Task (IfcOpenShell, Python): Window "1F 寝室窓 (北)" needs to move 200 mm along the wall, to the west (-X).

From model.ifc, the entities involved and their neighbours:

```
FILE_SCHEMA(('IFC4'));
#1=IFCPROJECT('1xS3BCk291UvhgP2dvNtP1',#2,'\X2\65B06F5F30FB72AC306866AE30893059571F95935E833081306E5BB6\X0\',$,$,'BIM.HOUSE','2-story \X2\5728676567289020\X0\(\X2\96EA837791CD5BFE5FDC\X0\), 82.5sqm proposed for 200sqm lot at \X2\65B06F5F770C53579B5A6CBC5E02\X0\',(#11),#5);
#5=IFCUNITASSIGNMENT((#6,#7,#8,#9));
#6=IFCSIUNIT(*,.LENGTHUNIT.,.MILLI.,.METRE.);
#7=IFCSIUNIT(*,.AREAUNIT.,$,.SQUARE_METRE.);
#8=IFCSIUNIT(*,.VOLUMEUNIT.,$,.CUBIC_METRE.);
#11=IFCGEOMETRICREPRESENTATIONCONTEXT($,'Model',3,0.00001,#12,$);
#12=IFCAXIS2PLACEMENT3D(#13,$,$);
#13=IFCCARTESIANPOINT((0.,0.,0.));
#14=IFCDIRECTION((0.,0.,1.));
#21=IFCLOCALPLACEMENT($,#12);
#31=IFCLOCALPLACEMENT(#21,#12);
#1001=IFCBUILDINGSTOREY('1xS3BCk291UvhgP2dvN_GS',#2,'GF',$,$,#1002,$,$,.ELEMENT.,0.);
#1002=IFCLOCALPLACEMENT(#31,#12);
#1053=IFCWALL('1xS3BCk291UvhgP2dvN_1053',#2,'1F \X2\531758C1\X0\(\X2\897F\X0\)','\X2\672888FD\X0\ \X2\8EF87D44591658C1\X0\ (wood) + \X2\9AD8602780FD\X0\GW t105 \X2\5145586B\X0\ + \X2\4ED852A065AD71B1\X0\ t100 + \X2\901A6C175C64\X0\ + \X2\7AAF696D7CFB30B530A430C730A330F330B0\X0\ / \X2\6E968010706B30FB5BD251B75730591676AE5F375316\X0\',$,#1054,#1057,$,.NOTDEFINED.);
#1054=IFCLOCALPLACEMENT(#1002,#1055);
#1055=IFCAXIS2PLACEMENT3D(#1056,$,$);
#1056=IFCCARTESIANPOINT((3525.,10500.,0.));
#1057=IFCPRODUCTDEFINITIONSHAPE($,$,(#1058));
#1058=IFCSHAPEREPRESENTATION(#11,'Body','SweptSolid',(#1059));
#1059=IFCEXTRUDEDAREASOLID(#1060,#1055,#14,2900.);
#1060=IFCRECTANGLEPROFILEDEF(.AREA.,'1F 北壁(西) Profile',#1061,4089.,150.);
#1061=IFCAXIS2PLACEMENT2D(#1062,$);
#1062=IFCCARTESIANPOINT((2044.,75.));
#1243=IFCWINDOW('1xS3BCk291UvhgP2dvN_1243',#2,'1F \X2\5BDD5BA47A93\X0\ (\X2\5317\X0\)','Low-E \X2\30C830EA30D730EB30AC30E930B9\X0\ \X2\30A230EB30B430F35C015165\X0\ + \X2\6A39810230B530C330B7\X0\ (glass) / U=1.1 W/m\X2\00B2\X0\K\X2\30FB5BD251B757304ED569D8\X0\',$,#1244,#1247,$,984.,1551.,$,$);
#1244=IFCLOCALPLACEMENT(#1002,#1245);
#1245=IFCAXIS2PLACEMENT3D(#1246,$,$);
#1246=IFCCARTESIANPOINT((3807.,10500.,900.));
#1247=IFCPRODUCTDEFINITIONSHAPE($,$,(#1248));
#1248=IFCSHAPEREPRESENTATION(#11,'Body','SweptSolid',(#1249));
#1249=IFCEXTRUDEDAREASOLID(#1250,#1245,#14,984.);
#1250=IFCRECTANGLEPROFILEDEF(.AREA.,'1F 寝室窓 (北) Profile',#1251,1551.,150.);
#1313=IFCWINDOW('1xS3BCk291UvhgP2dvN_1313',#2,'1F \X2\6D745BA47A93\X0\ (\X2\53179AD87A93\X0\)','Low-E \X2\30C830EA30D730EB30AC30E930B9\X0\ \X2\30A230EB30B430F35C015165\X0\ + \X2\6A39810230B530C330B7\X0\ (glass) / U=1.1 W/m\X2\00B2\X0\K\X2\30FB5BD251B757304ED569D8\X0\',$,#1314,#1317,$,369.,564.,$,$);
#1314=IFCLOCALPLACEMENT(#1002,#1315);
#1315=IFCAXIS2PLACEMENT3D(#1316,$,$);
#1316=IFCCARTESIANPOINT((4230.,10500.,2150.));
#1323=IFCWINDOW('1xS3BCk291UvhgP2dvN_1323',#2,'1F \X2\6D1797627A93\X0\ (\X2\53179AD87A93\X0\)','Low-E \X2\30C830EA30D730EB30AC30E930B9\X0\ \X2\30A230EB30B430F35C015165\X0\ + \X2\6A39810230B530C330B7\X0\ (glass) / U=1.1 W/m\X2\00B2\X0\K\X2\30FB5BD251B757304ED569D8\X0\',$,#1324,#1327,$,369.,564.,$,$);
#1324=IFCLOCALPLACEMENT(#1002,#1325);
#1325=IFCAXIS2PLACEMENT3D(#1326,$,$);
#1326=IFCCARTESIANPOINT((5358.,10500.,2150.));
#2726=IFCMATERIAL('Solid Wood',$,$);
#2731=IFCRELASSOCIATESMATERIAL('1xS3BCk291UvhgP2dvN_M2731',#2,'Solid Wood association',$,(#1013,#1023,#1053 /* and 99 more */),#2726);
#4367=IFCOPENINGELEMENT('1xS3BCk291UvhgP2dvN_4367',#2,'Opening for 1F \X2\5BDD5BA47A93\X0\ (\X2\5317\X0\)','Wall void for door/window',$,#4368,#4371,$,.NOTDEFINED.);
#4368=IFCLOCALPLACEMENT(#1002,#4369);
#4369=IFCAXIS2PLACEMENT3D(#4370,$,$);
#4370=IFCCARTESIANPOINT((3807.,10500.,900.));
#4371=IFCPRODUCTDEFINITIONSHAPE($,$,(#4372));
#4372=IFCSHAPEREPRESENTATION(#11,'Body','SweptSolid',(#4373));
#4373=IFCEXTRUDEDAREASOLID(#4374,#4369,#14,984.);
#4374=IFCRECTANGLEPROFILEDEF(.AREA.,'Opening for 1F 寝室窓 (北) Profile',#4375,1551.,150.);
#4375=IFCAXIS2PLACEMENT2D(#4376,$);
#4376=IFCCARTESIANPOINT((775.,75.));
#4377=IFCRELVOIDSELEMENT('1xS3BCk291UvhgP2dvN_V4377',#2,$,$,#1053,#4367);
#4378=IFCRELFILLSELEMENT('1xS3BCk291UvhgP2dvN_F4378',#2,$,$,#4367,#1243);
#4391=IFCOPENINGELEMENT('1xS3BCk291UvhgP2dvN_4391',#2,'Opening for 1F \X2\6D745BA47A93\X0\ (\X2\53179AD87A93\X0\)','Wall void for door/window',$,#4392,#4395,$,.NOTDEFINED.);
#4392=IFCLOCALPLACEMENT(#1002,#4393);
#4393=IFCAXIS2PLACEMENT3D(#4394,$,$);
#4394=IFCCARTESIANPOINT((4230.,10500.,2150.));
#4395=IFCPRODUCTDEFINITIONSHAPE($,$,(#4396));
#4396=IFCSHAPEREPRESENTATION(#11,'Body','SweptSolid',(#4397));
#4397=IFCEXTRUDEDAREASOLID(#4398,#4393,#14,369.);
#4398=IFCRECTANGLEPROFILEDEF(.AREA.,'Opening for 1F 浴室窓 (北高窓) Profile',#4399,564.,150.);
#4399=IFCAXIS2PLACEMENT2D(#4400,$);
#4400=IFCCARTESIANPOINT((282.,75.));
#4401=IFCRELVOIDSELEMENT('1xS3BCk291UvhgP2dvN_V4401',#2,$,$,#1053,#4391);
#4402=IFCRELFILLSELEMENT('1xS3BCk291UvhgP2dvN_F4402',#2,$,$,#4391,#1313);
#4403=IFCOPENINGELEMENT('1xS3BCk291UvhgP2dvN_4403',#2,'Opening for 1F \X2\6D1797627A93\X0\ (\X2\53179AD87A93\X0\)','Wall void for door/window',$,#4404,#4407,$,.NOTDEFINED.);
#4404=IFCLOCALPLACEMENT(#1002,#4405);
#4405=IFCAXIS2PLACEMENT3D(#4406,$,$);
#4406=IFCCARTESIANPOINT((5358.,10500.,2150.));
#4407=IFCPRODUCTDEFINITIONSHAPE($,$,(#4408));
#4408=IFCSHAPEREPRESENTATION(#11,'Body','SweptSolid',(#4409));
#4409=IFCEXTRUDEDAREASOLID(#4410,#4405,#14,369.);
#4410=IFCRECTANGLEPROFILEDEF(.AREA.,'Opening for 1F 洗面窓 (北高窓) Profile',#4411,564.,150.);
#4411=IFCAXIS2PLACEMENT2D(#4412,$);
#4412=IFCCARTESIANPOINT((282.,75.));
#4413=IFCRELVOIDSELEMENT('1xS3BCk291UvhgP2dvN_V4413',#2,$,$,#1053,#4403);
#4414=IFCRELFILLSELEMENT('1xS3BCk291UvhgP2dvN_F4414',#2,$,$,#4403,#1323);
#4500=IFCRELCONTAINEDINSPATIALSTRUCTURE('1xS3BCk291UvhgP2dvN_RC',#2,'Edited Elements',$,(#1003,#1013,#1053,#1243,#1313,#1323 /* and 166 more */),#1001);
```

```python
import ifcopenshell
import ifcopenshell.api.geometry
import ifcopenshell.util.placement
import ifcopenshell.util.unit

model = ifcopenshell.open("model.ifc")
unit_scale = ifcopenshell.util.unit.calculate_unit_scale(model)

window = model.by_guid("1xS3BCk291UvhgP2dvN_1243")
opening = window.FillsVoids[0].RelatingOpeningElement
wall = opening.VoidsElements[0].RelatingBuildingElement

wall_matrix = ifcopenshell.util.placement.get_local_placement(wall.ObjectPlacement)
shift = wall_matrix[:3, 0] * -0.2 / unit_scale
before = ifcopenshell.util.placement.get_local_placement(window.ObjectPlacement)[:3, 3].copy()

# The window is not placed relative to its opening, so move both.
for product in (opening, window):
    matrix = ifcopenshell.util.placement.get_local_placement(product.ObjectPlacement)
    matrix[:3, 3] += shift
    ifcopenshell.api.geometry.edit_object_placement(model, product=product, matrix=matrix, is_si=False)

after = ifcopenshell.util.placement.get_local_placement(window.ObjectPlacement)[:3, 3]
print("window moved by", (after - before).round(3) + 0.0)

model.write("model_edited.ifc")
```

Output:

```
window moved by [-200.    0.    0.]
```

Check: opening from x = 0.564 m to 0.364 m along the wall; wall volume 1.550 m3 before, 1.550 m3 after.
